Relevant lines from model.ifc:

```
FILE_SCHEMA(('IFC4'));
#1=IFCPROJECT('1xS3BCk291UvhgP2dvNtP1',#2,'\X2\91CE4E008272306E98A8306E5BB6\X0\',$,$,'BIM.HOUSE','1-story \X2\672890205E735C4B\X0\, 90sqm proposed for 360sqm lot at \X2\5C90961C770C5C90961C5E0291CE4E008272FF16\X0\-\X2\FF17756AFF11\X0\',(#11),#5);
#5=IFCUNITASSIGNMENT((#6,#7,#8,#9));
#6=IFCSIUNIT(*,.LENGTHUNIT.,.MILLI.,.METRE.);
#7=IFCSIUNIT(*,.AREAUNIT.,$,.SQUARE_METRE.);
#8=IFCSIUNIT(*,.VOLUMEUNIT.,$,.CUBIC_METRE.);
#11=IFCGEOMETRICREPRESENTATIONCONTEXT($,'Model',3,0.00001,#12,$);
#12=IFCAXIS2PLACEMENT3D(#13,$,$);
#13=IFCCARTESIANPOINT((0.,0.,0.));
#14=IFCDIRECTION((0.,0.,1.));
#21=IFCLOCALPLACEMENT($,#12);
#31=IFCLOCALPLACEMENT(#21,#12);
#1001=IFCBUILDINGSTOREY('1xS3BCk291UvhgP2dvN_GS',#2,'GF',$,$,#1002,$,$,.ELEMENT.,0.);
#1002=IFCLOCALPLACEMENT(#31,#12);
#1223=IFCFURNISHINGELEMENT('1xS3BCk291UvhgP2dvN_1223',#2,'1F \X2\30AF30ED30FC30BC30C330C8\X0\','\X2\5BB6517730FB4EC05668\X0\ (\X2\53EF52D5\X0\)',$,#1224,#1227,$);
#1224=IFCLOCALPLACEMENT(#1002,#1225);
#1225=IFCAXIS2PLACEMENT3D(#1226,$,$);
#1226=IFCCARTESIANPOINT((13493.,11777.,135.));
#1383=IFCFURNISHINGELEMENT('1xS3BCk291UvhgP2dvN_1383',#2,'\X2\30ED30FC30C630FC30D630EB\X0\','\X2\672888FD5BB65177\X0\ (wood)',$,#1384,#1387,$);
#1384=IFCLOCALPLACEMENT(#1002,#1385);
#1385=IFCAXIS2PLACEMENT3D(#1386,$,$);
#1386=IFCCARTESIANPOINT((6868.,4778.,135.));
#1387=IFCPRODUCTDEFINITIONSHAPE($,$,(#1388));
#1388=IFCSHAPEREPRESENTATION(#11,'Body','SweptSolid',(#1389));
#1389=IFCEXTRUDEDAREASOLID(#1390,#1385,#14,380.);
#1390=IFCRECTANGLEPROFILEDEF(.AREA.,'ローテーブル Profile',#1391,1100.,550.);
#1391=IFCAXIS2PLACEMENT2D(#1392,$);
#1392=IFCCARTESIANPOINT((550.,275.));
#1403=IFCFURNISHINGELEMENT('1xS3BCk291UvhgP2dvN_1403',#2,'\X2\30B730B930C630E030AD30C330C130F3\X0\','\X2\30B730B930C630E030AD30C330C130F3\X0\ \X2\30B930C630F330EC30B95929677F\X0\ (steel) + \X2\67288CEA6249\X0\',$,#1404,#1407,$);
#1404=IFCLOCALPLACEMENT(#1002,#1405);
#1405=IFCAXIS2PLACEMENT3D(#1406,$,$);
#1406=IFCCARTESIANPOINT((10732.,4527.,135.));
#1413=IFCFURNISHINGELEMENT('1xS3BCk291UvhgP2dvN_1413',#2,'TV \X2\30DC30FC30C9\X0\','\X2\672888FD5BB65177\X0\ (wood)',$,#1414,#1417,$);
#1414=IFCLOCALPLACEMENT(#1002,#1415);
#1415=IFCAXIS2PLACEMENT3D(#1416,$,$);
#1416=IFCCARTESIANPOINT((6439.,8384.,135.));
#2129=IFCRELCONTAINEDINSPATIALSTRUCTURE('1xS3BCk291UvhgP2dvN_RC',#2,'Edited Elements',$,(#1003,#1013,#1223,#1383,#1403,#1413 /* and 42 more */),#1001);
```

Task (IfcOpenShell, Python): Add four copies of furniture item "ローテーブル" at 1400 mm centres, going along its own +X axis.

```python
import ifcopenshell
import ifcopenshell.api.geometry
import ifcopenshell.api.root
import ifcopenshell.util.element
import ifcopenshell.util.placement
import ifcopenshell.util.unit

model = ifcopenshell.open("model.ifc")
unit_scale = ifcopenshell.util.unit.calculate_unit_scale(model)


def reuse_history(source, copy):
    """copy_class also copies each property set's owner history, people and application; keep the originals."""
    for rel in copy.IsDefinedBy:
        if rel.is_a("IfcRelDefinesByProperties") and (history := rel.RelatingPropertyDefinition.OwnerHistory):
            rel.RelatingPropertyDefinition.OwnerHistory = source.OwnerHistory
            ifcopenshell.util.element.remove_deep2(model, history)


source = model.by_id(1383)
base = ifcopenshell.util.placement.get_local_placement(source.ObjectPlacement)
step = base[:3, 0] * 1.4 / unit_scale

for i in range(1, 5):
    copy = ifcopenshell.api.root.copy_class(model, product=source)
    copy.Representation = ifcopenshell.util.element.copy_deep(
        model, source.Representation, exclude=["IfcGeometricRepresentationContext", "IfcRepresentationMap"]
    )
    reuse_history(source, copy)
    matrix = base.copy()
    matrix[:3, 3] += i * step
    print("added at", matrix[:3, 3].round(3) + 0.0)
    ifcopenshell.api.geometry.edit_object_placement(model, product=copy, matrix=matrix, is_si=False)

model.write("model_updated.ifc")
```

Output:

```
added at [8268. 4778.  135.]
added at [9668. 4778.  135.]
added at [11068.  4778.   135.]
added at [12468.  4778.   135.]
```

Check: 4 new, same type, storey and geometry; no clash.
